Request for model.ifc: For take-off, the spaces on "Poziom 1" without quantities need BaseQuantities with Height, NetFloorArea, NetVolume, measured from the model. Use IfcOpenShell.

First a look at what the model holds.

```python
import ifcopenshell
import ifcopenshell.util.element
import ifcopenshell.util.unit

model = ifcopenshell.open("model.ifc")
print(model.schema)
for unit_type in ("LENGTHUNIT", "AREAUNIT", "VOLUMEUNIT"):
    print(unit_type, ifcopenshell.util.unit.calculate_unit_scale(model, unit_type))
storey = next(s for s in model.by_type("IfcBuildingStorey") if s.Name == "Poziom 1")
spaces = [e for e in ifcopenshell.util.element.get_decomposition(storey) if e.is_a("IfcSpace")]
for e in sorted(spaces, key=lambda e: e.id()):
    print(e.id(), e.is_a(), e.Name, list(ifcopenshell.util.element.get_psets(e, qtos_only=True)), sep=" | ")
```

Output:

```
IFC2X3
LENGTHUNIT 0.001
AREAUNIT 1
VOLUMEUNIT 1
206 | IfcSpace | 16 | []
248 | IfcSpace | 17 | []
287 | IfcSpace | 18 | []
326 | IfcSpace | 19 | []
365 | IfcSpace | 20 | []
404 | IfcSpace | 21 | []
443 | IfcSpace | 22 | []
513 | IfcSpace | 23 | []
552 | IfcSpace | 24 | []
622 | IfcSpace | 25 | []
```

```python
import ifcopenshell
import ifcopenshell.api.pset
import ifcopenshell.geom
import ifcopenshell.util.element
import ifcopenshell.util.shape
import ifcopenshell.util.unit

model = ifcopenshell.open("model.ifc")
unit_scale = ifcopenshell.util.unit.calculate_unit_scale(model)
area_scale = ifcopenshell.util.unit.calculate_unit_scale(model, "AREAUNIT")
volume_scale = ifcopenshell.util.unit.calculate_unit_scale(model, "VOLUMEUNIT")
settings = ifcopenshell.geom.settings()

storey = next(s for s in model.by_type("IfcBuildingStorey") if s.Name == "Poziom 1")
spaces = [e for e in ifcopenshell.util.element.get_decomposition(storey) if e.is_a("IfcSpace")]

for e in sorted(spaces, key=lambda e: e.id()):
    if ifcopenshell.util.element.get_psets(e, qtos_only=True, should_inherit=False):
        continue
    # Geometry comes back in metres, in the element's own axes.
    shape = ifcopenshell.geom.create_shape(settings, e)
    values = {
        "Height": ifcopenshell.util.shape.get_z(shape.geometry) / unit_scale,
        "NetFloorArea": ifcopenshell.util.shape.get_footprint_area(shape.geometry) / area_scale,
        "NetVolume": ifcopenshell.util.shape.get_volume(shape.geometry) / volume_scale,
    }
    qto = ifcopenshell.api.pset.add_qto(model, product=e, name="BaseQuantities")
    ifcopenshell.api.pset.edit_qto(model, qto=qto, properties=values)
    print(e.id(), {k: round(v, 3) for k, v in values.items()})

model.write("model_rev.ifc")
```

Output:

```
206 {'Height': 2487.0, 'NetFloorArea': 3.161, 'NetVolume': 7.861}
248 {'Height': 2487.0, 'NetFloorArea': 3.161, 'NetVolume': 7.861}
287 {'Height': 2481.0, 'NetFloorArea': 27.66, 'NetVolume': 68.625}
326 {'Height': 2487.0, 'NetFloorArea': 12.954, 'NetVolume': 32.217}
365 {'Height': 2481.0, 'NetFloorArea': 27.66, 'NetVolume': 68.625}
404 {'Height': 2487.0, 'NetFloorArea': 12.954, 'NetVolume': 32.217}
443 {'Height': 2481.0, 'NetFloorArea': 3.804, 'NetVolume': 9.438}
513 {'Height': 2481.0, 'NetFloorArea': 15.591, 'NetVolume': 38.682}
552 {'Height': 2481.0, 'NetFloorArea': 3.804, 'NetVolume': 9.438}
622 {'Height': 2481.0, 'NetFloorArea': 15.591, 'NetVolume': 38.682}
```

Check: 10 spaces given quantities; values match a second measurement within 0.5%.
